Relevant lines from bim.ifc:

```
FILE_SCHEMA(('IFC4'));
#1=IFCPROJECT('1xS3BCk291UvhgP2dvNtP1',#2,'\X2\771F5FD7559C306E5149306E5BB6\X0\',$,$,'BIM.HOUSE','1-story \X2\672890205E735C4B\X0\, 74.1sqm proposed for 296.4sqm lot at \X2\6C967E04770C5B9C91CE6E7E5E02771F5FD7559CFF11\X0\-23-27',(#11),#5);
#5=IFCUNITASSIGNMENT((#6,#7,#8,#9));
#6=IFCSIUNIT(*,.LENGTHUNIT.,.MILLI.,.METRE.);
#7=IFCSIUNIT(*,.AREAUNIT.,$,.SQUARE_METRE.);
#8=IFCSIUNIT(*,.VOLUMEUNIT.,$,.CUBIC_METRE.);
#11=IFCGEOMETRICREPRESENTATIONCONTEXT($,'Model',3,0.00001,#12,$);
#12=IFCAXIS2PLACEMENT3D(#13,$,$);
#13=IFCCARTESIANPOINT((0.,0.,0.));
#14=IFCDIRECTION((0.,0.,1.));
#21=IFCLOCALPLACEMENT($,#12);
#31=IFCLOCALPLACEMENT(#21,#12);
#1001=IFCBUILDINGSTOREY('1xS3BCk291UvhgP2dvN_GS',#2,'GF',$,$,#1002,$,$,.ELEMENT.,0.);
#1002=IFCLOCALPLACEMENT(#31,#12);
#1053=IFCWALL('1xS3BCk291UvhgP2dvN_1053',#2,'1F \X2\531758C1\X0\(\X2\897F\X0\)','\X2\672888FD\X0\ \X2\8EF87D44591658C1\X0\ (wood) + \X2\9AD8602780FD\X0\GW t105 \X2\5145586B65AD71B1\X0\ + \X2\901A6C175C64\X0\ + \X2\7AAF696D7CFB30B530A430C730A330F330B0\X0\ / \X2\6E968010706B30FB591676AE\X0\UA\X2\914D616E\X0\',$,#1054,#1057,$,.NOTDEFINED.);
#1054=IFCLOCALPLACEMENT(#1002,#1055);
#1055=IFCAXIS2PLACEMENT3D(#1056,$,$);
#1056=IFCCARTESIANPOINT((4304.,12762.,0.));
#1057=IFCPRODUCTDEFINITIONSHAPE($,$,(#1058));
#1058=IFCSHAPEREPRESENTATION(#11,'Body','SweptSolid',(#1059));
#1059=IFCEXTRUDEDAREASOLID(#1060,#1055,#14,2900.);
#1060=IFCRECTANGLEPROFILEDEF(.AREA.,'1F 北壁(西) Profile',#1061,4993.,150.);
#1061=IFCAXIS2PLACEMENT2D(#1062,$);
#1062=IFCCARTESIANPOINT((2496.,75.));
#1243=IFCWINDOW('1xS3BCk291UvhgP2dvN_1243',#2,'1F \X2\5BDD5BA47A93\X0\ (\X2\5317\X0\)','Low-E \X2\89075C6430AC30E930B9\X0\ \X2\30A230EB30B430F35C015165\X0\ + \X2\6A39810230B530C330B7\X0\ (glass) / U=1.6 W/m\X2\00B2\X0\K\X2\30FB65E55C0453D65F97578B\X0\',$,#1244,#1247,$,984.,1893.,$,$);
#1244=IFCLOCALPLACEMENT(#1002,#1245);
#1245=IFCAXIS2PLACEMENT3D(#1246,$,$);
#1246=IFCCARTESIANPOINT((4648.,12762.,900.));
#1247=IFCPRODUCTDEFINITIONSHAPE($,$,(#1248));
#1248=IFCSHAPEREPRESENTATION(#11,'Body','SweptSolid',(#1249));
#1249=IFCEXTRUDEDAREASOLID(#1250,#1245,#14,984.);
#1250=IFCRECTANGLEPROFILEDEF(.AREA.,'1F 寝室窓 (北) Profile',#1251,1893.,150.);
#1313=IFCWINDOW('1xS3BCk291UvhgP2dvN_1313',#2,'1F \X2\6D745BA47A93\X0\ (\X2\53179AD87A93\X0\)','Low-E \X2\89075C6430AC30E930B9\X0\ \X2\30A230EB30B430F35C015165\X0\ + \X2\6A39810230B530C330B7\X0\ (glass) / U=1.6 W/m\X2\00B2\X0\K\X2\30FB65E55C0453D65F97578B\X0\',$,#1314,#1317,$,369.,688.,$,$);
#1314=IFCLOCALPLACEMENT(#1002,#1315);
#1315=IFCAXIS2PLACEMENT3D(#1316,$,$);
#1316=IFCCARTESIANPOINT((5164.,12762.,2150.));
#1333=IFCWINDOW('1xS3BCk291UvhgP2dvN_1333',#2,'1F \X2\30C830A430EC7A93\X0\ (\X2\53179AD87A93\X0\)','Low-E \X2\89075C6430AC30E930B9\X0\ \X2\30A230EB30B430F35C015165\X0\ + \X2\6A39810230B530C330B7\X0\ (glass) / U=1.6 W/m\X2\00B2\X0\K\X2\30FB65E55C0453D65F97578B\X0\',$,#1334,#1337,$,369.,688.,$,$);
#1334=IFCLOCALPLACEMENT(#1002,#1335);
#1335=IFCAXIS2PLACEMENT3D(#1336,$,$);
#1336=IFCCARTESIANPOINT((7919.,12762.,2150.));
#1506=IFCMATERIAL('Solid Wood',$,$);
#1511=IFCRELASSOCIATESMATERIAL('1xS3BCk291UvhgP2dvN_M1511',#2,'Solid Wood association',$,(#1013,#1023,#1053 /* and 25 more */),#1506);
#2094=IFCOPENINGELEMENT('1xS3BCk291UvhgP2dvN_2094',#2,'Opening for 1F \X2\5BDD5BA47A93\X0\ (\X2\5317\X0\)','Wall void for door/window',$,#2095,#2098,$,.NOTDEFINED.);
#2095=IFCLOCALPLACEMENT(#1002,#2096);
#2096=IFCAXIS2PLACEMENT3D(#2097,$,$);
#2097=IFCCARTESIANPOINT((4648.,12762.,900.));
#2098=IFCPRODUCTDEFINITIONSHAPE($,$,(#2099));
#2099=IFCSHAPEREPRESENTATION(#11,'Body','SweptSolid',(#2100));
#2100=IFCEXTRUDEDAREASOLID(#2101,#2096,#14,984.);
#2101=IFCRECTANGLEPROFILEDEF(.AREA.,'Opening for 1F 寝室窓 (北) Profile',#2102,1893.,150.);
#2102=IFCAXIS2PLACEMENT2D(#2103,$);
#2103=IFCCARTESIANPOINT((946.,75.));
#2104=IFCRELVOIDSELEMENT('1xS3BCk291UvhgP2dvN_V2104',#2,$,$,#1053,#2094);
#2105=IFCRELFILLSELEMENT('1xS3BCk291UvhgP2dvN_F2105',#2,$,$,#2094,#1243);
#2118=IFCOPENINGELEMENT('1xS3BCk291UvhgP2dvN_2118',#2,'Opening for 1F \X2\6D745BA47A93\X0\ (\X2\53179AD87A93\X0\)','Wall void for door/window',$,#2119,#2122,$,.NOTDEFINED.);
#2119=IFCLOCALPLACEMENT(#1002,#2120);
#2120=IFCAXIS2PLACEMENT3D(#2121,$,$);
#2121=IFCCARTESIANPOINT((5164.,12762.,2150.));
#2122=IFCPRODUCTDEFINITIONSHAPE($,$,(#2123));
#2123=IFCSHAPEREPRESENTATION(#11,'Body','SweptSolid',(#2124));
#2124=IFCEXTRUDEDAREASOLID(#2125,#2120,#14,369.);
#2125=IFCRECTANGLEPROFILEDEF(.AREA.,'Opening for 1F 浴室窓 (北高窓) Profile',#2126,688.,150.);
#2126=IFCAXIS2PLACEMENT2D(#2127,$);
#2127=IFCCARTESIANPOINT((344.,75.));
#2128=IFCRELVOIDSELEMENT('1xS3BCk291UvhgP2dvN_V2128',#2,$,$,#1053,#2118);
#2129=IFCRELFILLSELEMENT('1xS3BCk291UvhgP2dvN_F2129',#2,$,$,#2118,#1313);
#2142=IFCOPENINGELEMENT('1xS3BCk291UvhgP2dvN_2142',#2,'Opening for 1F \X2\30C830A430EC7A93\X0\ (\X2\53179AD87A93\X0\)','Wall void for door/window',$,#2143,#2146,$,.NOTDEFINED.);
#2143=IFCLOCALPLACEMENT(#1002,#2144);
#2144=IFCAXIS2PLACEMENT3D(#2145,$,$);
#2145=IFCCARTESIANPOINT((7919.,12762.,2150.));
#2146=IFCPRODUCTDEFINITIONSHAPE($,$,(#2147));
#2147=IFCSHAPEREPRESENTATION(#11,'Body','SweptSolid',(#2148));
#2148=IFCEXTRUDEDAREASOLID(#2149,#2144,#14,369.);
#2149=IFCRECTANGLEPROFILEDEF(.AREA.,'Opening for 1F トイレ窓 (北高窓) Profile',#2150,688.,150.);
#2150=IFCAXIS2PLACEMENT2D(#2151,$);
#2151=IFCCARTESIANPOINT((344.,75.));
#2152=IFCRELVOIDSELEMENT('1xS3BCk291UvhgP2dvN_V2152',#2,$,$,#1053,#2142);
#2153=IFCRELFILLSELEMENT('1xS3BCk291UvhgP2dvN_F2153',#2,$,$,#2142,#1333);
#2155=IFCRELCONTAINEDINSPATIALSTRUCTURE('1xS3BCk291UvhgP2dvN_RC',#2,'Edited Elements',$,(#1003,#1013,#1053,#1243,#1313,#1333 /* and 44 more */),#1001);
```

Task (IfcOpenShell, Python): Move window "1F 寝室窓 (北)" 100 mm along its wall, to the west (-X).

```python
import ifcopenshell
import ifcopenshell.api.geometry
import ifcopenshell.util.placement
import ifcopenshell.util.unit

model = ifcopenshell.open("bim.ifc")
unit_scale = ifcopenshell.util.unit.calculate_unit_scale(model)

window = model.by_guid("1xS3BCk291UvhgP2dvN_1243")
opening = window.FillsVoids[0].RelatingOpeningElement
wall = opening.VoidsElements[0].RelatingBuildingElement

wall_matrix = ifcopenshell.util.placement.get_local_placement(wall.ObjectPlacement)
shift = wall_matrix[:3, 0] * -0.1 / unit_scale
before = ifcopenshell.util.placement.get_local_placement(window.ObjectPlacement)[:3, 3].copy()

# The window is not placed relative to its opening, so move both.
for product in (opening, window):
    matrix = ifcopenshell.util.placement.get_local_placement(product.ObjectPlacement)
    matrix[:3, 3] += shift
    ifcopenshell.api.geometry.edit_object_placement(model, product=product, matrix=matrix, is_si=False)

after = ifcopenshell.util.placement.get_local_placement(window.ObjectPlacement)[:3, 3]
print("window moved by", (after - before).round(3) + 0.0)

model.write("bim_v2.ifc")
```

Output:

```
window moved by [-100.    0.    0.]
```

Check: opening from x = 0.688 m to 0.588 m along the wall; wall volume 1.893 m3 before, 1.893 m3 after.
